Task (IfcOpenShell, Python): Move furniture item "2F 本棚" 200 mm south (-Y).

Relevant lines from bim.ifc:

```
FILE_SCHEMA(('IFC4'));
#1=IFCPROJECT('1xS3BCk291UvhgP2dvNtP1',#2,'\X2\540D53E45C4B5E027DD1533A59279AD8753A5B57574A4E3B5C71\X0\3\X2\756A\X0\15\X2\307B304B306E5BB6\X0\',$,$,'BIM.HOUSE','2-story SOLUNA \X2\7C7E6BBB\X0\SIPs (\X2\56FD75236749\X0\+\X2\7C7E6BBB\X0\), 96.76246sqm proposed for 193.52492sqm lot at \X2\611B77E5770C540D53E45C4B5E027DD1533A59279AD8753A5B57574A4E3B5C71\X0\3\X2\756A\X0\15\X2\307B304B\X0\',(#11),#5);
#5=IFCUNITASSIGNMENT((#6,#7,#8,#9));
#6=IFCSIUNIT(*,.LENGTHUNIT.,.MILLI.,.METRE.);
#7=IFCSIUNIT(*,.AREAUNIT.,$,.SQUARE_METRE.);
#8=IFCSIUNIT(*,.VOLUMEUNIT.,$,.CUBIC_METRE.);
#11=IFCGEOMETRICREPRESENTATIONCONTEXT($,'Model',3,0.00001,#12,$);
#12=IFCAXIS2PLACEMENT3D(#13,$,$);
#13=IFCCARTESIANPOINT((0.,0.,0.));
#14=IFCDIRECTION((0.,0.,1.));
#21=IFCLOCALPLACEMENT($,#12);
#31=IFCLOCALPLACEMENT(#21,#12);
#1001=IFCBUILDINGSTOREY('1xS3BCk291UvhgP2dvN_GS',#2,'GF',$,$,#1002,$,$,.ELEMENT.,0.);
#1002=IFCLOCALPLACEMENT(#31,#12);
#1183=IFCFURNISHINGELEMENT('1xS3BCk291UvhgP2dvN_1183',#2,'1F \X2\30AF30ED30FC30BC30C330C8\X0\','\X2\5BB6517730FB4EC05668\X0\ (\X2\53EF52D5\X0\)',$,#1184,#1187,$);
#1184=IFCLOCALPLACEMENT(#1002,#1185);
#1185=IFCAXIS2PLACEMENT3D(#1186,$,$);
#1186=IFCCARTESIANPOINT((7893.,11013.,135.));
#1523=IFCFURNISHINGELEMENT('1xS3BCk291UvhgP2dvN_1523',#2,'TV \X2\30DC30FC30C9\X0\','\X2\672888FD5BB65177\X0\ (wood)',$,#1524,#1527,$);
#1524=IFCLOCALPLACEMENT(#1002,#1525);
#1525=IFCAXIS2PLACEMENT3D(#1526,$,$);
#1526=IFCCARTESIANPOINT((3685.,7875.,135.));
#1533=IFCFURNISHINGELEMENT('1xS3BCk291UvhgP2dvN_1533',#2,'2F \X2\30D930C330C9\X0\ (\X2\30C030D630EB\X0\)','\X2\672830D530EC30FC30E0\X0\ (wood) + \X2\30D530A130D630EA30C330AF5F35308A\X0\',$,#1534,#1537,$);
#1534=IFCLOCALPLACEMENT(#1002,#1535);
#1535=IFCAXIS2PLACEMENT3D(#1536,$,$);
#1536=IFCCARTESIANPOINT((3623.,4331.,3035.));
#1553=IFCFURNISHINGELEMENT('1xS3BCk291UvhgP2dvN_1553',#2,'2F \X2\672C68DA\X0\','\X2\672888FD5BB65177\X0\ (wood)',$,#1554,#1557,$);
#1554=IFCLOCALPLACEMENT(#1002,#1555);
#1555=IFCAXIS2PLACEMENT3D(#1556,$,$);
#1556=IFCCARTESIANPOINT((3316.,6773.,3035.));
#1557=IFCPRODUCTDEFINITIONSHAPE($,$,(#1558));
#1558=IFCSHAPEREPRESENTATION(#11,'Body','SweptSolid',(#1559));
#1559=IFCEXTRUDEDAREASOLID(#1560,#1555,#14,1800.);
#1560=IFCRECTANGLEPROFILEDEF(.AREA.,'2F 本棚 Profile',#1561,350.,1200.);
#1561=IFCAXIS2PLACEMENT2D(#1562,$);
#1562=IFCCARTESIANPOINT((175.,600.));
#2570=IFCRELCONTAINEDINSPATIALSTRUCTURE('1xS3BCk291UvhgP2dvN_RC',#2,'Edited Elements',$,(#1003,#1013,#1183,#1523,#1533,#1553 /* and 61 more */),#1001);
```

```python
import ifcopenshell
import ifcopenshell.api.geometry
import ifcopenshell.util.placement

model = ifcopenshell.open("bim.ifc")

item = model.by_guid("1xS3BCk291UvhgP2dvN_1553")
matrix = ifcopenshell.util.placement.get_local_placement(item.ObjectPlacement)
matrix[1, 3] -= 200.0
ifcopenshell.api.geometry.edit_object_placement(model, product=item, matrix=matrix, is_si=False)

print(ifcopenshell.util.placement.get_local_placement(item.ObjectPlacement).round(3) + 0.0)

model.write("bim_rev.ifc")
```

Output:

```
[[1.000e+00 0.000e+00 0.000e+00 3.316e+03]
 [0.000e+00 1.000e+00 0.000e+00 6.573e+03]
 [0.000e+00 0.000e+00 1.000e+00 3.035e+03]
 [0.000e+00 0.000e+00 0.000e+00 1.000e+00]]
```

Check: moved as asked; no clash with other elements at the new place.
